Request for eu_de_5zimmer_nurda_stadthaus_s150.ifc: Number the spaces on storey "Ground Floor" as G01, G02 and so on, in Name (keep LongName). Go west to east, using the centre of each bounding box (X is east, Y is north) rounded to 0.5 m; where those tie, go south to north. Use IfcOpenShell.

First a look at what the model holds.

```python
import ifcopenshell
import ifcopenshell.util.element
import ifcopenshell.util.placement

model = ifcopenshell.open("eu_de_5zimmer_nurda_stadthaus_s150.ifc")
print(model.schema)
storey = next(s for s in model.by_type("IfcBuildingStorey") if s.Name == "Ground Floor")
spaces = [e for e in ifcopenshell.util.element.get_decomposition(storey) if e.is_a("IfcSpace")]
for e in sorted(spaces, key=lambda e: e.id()):
    origin = ifcopenshell.util.placement.get_local_placement(e.ObjectPlacement)[:3, 3]
    print(e.id(), e.Name, e.LongName, origin.round(2) + 0.0, sep=" | ")
```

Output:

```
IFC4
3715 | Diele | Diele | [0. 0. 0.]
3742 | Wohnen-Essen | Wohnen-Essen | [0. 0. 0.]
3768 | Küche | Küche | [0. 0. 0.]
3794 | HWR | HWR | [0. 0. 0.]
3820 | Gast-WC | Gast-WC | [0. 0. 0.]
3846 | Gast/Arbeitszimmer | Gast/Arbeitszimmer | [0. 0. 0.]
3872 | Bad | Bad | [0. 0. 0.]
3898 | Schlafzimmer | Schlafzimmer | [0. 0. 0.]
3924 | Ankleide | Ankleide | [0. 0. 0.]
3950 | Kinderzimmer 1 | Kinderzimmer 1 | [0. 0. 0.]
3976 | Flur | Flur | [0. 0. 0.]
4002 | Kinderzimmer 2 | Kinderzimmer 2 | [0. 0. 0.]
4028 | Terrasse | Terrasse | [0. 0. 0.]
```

```python
import ifcopenshell
import ifcopenshell.geom
import ifcopenshell.util.element
import ifcopenshell.util.shape

model = ifcopenshell.open("eu_de_5zimmer_nurda_stadthaus_s150.ifc")
settings = ifcopenshell.geom.settings()
settings.set("use-world-coords", True)


def centre(element):
    shape = ifcopenshell.geom.create_shape(settings, element)
    return ifcopenshell.util.shape.get_bbox_centroid(shape.geometry)


storey = next(s for s in model.by_type("IfcBuildingStorey") if s.Name == "Ground Floor")
spaces = [e for e in ifcopenshell.util.element.get_decomposition(storey) if e.is_a("IfcSpace")]

# Insertion points can sit at a corner or the storey origin, so sort by the geometry (in metres).
centres = {e: centre(e) for e in spaces}
spaces.sort(key=lambda e: (round(centres[e][0] / 0.5), centres[e][1]))

for i, e in enumerate(spaces, start=1):
    number = f"G{i:02d}"
    e.Name = number
    print(e.id(), number)

model.write("eu_de_5zimmer_nurda_stadthaus_s150_updated.ifc")
```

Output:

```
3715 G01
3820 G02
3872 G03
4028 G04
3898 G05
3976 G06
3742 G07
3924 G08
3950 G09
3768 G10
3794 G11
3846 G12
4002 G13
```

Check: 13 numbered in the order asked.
